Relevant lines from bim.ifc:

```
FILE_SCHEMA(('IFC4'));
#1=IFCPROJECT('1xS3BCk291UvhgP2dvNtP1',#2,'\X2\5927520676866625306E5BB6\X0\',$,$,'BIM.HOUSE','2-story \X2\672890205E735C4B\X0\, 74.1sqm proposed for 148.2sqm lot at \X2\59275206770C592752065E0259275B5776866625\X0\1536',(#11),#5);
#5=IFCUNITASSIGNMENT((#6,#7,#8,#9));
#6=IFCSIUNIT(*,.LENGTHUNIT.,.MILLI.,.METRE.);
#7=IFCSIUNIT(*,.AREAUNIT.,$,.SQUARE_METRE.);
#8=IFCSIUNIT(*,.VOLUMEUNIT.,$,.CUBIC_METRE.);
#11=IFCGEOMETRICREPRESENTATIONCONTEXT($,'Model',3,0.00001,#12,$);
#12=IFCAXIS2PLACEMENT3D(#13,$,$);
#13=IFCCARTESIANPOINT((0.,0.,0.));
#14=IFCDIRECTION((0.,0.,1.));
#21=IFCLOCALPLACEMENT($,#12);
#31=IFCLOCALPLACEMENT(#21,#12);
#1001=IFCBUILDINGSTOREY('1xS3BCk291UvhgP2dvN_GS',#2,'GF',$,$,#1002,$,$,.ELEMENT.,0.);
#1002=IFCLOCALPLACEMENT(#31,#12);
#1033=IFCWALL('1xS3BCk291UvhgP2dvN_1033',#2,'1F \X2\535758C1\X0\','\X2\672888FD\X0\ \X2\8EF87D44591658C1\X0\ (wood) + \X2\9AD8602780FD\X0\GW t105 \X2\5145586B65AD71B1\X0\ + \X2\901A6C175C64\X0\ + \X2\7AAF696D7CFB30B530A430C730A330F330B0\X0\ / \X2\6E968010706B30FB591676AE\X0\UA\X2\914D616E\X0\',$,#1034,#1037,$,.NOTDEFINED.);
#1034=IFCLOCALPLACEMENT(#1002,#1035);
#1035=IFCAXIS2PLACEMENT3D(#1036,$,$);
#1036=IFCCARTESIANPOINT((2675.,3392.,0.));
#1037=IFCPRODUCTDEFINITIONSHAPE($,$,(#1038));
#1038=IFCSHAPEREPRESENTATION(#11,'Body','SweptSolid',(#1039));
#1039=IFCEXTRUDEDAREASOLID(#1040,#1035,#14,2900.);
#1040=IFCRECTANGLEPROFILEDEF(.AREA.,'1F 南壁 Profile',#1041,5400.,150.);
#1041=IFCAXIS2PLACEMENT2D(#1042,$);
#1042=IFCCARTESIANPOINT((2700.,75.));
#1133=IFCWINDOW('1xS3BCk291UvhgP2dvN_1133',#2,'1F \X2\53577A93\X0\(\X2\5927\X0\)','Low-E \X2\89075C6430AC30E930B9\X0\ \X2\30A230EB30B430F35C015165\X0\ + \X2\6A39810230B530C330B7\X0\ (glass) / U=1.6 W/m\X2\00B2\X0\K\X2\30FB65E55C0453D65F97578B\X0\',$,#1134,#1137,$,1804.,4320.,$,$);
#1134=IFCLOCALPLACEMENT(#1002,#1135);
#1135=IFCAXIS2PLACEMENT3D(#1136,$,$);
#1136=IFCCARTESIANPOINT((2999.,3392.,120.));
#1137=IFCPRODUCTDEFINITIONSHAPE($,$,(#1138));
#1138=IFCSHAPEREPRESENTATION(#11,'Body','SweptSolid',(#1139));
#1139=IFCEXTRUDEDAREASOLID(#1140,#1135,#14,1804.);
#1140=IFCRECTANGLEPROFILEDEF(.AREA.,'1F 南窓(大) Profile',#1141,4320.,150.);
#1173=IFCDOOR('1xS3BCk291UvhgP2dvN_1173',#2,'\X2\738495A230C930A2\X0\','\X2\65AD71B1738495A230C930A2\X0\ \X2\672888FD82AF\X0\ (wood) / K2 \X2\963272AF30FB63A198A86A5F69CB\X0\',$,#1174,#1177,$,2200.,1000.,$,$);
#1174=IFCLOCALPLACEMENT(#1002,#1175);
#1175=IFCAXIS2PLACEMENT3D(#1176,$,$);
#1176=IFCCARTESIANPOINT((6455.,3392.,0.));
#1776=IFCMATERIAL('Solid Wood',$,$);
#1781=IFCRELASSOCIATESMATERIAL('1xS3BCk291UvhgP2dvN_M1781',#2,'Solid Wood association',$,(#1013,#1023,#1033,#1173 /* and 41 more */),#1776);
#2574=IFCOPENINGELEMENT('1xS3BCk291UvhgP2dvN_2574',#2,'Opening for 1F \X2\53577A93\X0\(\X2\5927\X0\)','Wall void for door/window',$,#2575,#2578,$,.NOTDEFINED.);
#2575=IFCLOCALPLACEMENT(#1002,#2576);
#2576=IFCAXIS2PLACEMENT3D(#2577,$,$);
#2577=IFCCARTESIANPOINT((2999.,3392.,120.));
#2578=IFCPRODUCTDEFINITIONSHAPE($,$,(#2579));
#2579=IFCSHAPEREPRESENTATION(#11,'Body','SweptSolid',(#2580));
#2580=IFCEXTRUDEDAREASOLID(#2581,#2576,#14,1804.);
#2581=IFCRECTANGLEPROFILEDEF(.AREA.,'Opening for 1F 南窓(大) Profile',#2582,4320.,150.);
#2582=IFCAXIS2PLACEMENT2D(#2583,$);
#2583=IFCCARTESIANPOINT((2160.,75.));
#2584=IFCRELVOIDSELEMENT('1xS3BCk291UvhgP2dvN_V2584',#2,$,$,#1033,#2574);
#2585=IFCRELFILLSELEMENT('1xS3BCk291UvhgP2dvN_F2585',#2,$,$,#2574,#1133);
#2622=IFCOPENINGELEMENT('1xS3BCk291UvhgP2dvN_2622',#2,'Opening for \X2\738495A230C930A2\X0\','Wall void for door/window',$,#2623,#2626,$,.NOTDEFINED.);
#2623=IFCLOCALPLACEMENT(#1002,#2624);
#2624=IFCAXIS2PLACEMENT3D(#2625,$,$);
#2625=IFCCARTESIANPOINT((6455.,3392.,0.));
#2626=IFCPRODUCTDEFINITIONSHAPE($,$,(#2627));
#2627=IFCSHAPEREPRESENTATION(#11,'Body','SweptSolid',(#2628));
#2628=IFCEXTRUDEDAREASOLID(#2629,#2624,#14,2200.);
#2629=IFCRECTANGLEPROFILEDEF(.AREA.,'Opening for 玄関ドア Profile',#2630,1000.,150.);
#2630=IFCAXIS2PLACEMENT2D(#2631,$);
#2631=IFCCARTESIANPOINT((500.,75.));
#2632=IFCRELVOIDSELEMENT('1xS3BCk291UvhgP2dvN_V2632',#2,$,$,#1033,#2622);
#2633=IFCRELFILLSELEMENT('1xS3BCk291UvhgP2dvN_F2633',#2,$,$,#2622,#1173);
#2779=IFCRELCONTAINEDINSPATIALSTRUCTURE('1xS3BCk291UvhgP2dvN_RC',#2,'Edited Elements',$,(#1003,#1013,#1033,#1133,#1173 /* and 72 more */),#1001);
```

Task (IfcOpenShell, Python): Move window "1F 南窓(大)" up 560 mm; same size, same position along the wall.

```python
import numpy as np
import ifcopenshell
import ifcopenshell.api.geometry
import ifcopenshell.util.placement
import ifcopenshell.util.unit

model = ifcopenshell.open("bim.ifc")
unit_scale = ifcopenshell.util.unit.calculate_unit_scale(model)

window = model.by_guid("1xS3BCk291UvhgP2dvN_1133")
opening = window.FillsVoids[0].RelatingOpeningElement
dz = 0.56 / unit_scale

shift = np.array([0.0, 0.0, dz])
# The window is not placed relative to its opening, so move both.
for product in (opening, window):
    matrix = ifcopenshell.util.placement.get_local_placement(product.ObjectPlacement)
    matrix[:3, 3] += shift
    ifcopenshell.api.geometry.edit_object_placement(model, product=product, matrix=matrix, is_si=False)

print(f"moved by {dz * unit_scale:+.3f} m")

model.write("bim_edited.ifc")
```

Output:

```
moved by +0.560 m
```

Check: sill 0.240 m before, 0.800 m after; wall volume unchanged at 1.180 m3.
